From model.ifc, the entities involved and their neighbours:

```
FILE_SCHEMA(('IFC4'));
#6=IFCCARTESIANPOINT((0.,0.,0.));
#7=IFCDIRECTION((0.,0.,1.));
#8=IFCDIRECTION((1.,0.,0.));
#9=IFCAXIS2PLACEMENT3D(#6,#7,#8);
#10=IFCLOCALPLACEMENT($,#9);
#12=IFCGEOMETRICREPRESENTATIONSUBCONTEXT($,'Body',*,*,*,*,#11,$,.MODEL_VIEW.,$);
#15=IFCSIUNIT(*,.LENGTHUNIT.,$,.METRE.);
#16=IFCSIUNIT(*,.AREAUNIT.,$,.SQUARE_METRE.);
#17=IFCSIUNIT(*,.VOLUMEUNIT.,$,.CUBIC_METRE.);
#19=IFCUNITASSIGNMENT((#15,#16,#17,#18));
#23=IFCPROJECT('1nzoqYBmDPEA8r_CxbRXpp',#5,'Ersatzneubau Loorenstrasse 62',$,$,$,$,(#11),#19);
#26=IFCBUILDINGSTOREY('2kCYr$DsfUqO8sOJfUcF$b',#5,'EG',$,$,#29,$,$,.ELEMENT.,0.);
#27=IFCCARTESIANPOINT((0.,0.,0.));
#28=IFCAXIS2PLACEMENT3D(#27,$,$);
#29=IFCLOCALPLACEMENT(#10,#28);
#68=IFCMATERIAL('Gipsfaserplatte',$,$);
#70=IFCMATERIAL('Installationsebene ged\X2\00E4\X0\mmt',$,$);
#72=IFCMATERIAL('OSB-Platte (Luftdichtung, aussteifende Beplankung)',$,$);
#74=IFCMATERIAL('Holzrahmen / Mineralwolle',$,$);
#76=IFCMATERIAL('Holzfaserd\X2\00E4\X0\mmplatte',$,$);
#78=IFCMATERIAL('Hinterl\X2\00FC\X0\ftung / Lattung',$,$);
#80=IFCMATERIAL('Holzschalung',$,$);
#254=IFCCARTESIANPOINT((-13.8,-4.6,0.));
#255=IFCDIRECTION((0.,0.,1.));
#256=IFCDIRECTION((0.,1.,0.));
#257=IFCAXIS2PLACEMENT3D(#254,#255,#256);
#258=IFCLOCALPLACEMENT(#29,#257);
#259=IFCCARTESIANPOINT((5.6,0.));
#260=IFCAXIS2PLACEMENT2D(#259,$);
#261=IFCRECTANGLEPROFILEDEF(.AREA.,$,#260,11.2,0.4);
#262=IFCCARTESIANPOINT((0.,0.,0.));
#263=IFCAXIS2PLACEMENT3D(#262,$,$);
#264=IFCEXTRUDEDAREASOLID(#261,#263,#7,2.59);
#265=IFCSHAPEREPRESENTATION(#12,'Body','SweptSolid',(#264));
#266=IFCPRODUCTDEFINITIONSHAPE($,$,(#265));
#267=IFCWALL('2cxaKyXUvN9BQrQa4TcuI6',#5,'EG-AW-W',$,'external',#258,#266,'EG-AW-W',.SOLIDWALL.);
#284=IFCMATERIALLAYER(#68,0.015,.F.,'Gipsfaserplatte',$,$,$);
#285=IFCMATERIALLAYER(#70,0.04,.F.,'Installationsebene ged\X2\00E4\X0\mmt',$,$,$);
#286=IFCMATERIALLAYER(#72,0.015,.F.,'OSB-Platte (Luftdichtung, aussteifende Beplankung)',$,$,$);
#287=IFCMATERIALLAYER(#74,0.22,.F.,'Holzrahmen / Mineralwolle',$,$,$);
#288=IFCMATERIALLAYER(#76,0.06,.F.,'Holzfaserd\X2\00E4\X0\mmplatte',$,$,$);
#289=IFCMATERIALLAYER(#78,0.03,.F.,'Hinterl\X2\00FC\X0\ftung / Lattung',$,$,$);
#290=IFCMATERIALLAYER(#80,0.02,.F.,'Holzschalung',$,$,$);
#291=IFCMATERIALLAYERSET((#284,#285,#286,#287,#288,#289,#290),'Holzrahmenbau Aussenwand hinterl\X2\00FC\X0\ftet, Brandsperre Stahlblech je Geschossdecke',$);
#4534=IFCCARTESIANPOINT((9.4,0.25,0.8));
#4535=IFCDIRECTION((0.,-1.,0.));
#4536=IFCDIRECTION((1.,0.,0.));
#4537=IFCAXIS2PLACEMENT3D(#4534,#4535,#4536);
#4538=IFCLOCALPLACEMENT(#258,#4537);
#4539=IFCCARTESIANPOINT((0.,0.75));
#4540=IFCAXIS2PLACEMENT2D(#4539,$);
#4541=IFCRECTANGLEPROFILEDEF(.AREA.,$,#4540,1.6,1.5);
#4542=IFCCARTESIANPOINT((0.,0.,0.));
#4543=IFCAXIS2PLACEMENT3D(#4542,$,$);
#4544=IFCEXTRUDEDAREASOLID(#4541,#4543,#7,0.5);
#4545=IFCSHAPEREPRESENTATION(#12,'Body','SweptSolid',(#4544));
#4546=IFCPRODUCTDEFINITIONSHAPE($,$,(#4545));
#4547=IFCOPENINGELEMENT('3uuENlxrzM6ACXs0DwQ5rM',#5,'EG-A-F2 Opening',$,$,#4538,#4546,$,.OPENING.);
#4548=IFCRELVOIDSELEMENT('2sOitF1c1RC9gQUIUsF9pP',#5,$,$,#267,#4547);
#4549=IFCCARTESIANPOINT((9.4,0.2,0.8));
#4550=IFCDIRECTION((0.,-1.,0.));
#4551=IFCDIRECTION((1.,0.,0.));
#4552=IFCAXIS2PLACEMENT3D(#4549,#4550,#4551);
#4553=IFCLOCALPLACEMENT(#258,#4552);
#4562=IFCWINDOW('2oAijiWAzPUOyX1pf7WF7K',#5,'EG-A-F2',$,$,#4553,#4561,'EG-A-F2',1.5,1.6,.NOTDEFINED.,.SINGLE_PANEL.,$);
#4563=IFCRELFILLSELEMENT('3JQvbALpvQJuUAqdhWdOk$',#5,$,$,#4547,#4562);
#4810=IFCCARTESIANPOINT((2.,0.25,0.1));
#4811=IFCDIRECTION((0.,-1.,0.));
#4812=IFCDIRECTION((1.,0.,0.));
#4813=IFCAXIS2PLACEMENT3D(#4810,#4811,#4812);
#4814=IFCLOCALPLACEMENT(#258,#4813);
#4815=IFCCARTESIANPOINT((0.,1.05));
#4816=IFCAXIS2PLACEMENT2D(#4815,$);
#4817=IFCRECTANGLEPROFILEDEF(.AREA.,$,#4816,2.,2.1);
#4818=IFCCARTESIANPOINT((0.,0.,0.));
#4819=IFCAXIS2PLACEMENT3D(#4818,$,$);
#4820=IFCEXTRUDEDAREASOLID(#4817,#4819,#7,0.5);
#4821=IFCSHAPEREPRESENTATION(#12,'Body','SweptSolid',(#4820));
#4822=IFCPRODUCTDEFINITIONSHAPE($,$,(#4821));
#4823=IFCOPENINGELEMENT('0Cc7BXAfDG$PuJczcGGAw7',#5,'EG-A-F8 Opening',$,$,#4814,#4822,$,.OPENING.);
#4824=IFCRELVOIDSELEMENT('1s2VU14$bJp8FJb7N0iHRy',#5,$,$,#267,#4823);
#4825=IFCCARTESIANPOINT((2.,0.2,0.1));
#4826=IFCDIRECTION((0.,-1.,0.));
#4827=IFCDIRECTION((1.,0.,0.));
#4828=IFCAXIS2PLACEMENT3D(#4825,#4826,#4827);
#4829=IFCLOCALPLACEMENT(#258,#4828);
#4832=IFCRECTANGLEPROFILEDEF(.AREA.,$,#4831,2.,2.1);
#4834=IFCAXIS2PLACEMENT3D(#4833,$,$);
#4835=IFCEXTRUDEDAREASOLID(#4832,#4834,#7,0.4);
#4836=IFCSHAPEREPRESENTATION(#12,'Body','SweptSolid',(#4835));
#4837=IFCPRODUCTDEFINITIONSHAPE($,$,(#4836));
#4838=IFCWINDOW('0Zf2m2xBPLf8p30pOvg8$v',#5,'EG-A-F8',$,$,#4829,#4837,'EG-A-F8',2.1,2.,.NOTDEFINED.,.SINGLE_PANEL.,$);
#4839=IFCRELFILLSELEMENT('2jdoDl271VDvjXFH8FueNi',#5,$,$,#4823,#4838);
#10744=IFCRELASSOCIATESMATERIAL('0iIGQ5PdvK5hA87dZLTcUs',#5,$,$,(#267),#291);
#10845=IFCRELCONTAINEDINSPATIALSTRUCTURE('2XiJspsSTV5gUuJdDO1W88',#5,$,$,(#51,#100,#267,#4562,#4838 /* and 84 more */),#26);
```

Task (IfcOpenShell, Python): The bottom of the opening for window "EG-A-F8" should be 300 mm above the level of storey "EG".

```python
import numpy as np
import ifcopenshell
import ifcopenshell.api.geometry
import ifcopenshell.geom
import ifcopenshell.util.element
import ifcopenshell.util.placement
import ifcopenshell.util.shape
import ifcopenshell.util.unit

model = ifcopenshell.open("model.ifc")
unit_scale = ifcopenshell.util.unit.calculate_unit_scale(model)

window = model.by_id(4838)
opening = window.FillsVoids[0].RelatingOpeningElement
storey = ifcopenshell.util.element.get_container(window, ifc_class="IfcBuildingStorey")
level = ifcopenshell.util.placement.get_local_placement(storey.ObjectPlacement)[2, 3]

# The opening's origin need not be at the sill, so measure its lowest point.
shape = ifcopenshell.geom.create_shape(ifcopenshell.geom.settings(), opening)
bottom = ifcopenshell.util.shape.get_shape_bottom_elevation(shape, shape.geometry) / unit_scale
dz = level + 0.3 - bottom

shift = np.array([0.0, 0.0, dz])
# The window is not placed relative to its opening, so move both.
for product in (opening, window):
    matrix = ifcopenshell.util.placement.get_local_placement(product.ObjectPlacement)
    matrix[:3, 3] += shift
    ifcopenshell.api.geometry.edit_object_placement(model, product=product, matrix=matrix, is_si=False)

print(f"moved by {dz * unit_scale:+.3f} m")

model.write("model_edited.ifc")
```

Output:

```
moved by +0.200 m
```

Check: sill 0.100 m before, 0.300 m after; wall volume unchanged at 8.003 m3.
